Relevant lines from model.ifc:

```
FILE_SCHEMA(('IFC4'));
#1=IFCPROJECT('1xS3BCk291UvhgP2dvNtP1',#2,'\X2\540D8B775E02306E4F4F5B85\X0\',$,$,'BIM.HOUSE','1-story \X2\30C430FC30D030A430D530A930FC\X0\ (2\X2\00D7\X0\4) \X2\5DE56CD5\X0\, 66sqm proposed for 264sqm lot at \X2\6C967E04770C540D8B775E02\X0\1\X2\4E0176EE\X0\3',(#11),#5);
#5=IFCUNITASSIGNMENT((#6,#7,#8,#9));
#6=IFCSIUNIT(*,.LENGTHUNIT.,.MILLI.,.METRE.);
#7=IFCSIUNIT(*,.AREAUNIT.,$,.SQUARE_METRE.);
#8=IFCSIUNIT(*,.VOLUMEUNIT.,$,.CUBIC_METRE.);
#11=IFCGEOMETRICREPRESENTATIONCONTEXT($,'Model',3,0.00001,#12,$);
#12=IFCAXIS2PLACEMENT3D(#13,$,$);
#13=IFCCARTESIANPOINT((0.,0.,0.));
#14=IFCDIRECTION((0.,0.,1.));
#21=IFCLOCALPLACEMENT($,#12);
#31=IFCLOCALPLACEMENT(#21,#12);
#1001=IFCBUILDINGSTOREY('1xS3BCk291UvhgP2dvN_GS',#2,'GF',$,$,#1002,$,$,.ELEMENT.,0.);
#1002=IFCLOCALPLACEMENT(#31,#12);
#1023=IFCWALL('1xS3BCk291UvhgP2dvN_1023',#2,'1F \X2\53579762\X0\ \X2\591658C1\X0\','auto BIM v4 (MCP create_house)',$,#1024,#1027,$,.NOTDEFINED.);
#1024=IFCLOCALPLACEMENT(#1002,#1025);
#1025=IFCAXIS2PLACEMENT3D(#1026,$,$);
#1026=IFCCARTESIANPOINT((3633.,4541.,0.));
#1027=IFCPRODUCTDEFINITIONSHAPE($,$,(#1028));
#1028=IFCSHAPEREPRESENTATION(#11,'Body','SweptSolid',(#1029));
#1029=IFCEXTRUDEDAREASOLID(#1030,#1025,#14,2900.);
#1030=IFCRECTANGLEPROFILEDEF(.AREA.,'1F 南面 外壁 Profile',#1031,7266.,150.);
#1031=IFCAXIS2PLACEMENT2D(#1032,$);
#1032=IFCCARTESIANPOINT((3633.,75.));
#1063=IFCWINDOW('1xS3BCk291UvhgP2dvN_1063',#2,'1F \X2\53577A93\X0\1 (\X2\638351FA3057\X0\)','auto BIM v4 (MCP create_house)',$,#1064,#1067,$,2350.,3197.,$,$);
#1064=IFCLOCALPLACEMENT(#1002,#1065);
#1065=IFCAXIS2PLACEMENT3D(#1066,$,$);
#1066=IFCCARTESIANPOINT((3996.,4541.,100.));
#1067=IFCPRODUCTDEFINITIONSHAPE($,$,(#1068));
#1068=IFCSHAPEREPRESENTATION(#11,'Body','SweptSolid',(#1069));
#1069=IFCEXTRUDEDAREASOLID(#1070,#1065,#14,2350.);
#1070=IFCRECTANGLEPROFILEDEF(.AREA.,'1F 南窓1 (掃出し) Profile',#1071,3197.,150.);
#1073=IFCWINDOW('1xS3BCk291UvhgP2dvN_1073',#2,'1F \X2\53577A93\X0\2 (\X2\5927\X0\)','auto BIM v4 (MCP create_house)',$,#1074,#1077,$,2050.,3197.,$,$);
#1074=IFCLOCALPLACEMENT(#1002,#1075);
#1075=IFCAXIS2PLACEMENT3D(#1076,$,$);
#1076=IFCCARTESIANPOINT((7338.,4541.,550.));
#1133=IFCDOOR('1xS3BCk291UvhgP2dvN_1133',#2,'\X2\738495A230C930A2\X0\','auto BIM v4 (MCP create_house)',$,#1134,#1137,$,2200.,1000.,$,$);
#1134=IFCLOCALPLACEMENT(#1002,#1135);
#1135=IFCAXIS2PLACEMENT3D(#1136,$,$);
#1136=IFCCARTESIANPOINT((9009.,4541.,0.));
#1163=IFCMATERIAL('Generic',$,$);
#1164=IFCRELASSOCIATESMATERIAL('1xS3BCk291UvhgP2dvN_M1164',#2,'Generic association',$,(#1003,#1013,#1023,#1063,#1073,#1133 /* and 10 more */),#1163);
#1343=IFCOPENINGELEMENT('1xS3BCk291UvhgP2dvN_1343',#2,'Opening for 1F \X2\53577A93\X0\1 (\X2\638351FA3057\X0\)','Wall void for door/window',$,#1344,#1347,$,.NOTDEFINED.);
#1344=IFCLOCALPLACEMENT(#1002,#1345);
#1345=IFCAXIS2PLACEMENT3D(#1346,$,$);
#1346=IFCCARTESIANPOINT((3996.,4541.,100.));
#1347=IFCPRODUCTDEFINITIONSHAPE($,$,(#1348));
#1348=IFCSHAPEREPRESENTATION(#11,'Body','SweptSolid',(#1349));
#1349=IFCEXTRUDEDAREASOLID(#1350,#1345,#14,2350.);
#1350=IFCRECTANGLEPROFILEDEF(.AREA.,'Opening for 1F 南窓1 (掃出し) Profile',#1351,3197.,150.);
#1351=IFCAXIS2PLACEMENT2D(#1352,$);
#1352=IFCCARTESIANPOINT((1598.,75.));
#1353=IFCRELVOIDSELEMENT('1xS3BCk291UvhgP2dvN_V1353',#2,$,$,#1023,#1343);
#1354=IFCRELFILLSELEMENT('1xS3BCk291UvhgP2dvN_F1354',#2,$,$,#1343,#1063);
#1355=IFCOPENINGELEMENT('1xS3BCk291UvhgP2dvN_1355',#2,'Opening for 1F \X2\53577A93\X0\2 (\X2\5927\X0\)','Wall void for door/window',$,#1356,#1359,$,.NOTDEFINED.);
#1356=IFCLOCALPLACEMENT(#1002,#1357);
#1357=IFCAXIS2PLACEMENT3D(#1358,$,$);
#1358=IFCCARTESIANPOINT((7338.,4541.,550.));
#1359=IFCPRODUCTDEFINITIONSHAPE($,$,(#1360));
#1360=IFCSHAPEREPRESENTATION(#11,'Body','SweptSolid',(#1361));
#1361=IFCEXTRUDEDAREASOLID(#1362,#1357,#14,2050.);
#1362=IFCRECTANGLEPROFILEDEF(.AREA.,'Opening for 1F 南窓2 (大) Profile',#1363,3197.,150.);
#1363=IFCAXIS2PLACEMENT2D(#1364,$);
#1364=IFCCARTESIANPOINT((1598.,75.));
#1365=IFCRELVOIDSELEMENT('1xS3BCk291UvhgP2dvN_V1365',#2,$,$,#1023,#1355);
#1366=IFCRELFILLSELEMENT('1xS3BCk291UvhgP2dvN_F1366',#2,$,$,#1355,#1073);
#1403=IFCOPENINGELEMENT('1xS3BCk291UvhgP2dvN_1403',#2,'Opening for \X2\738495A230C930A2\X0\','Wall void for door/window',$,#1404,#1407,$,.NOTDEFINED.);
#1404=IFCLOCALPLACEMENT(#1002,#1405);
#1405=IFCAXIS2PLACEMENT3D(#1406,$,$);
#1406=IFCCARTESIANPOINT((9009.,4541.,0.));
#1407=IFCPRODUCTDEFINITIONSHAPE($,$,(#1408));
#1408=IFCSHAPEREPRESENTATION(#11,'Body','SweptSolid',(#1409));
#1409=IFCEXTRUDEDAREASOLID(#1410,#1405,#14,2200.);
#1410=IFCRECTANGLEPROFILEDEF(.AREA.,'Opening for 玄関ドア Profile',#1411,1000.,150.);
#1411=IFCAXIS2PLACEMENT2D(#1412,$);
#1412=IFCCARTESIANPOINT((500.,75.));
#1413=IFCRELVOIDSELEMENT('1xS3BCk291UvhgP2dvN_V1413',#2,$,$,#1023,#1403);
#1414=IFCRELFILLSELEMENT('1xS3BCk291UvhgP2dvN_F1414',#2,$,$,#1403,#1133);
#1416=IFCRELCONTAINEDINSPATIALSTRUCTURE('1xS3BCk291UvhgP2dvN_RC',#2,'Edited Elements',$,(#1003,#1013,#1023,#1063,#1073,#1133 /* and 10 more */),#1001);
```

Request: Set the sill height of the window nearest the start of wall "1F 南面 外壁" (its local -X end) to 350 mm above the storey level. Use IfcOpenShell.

```python
import numpy as np
import ifcopenshell
import ifcopenshell.api.geometry
import ifcopenshell.geom
import ifcopenshell.util.element
import ifcopenshell.util.placement
import ifcopenshell.util.shape
import ifcopenshell.util.unit

model = ifcopenshell.open("model.ifc")
unit_scale = ifcopenshell.util.unit.calculate_unit_scale(model)

window = model.by_id(1063)
opening = window.FillsVoids[0].RelatingOpeningElement
storey = ifcopenshell.util.element.get_container(window, ifc_class="IfcBuildingStorey")
level = ifcopenshell.util.placement.get_local_placement(storey.ObjectPlacement)[2, 3]

# The opening's origin need not be at the sill, so measure its lowest point.
shape = ifcopenshell.geom.create_shape(ifcopenshell.geom.settings(), opening)
bottom = ifcopenshell.util.shape.get_shape_bottom_elevation(shape, shape.geometry) / unit_scale
dz = level + 350.0 - bottom

shift = np.array([0.0, 0.0, dz])
# The window is not placed relative to its opening, so move both.
for product in (opening, window):
    matrix = ifcopenshell.util.placement.get_local_placement(product.ObjectPlacement)
    matrix[:3, 3] += shift
    ifcopenshell.api.geometry.edit_object_placement(model, product=product, matrix=matrix, is_si=False)

print(f"moved by {dz * unit_scale:+.3f} m")

model.write("model_updated.ifc")
```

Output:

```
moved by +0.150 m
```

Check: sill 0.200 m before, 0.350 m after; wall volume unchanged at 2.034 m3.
